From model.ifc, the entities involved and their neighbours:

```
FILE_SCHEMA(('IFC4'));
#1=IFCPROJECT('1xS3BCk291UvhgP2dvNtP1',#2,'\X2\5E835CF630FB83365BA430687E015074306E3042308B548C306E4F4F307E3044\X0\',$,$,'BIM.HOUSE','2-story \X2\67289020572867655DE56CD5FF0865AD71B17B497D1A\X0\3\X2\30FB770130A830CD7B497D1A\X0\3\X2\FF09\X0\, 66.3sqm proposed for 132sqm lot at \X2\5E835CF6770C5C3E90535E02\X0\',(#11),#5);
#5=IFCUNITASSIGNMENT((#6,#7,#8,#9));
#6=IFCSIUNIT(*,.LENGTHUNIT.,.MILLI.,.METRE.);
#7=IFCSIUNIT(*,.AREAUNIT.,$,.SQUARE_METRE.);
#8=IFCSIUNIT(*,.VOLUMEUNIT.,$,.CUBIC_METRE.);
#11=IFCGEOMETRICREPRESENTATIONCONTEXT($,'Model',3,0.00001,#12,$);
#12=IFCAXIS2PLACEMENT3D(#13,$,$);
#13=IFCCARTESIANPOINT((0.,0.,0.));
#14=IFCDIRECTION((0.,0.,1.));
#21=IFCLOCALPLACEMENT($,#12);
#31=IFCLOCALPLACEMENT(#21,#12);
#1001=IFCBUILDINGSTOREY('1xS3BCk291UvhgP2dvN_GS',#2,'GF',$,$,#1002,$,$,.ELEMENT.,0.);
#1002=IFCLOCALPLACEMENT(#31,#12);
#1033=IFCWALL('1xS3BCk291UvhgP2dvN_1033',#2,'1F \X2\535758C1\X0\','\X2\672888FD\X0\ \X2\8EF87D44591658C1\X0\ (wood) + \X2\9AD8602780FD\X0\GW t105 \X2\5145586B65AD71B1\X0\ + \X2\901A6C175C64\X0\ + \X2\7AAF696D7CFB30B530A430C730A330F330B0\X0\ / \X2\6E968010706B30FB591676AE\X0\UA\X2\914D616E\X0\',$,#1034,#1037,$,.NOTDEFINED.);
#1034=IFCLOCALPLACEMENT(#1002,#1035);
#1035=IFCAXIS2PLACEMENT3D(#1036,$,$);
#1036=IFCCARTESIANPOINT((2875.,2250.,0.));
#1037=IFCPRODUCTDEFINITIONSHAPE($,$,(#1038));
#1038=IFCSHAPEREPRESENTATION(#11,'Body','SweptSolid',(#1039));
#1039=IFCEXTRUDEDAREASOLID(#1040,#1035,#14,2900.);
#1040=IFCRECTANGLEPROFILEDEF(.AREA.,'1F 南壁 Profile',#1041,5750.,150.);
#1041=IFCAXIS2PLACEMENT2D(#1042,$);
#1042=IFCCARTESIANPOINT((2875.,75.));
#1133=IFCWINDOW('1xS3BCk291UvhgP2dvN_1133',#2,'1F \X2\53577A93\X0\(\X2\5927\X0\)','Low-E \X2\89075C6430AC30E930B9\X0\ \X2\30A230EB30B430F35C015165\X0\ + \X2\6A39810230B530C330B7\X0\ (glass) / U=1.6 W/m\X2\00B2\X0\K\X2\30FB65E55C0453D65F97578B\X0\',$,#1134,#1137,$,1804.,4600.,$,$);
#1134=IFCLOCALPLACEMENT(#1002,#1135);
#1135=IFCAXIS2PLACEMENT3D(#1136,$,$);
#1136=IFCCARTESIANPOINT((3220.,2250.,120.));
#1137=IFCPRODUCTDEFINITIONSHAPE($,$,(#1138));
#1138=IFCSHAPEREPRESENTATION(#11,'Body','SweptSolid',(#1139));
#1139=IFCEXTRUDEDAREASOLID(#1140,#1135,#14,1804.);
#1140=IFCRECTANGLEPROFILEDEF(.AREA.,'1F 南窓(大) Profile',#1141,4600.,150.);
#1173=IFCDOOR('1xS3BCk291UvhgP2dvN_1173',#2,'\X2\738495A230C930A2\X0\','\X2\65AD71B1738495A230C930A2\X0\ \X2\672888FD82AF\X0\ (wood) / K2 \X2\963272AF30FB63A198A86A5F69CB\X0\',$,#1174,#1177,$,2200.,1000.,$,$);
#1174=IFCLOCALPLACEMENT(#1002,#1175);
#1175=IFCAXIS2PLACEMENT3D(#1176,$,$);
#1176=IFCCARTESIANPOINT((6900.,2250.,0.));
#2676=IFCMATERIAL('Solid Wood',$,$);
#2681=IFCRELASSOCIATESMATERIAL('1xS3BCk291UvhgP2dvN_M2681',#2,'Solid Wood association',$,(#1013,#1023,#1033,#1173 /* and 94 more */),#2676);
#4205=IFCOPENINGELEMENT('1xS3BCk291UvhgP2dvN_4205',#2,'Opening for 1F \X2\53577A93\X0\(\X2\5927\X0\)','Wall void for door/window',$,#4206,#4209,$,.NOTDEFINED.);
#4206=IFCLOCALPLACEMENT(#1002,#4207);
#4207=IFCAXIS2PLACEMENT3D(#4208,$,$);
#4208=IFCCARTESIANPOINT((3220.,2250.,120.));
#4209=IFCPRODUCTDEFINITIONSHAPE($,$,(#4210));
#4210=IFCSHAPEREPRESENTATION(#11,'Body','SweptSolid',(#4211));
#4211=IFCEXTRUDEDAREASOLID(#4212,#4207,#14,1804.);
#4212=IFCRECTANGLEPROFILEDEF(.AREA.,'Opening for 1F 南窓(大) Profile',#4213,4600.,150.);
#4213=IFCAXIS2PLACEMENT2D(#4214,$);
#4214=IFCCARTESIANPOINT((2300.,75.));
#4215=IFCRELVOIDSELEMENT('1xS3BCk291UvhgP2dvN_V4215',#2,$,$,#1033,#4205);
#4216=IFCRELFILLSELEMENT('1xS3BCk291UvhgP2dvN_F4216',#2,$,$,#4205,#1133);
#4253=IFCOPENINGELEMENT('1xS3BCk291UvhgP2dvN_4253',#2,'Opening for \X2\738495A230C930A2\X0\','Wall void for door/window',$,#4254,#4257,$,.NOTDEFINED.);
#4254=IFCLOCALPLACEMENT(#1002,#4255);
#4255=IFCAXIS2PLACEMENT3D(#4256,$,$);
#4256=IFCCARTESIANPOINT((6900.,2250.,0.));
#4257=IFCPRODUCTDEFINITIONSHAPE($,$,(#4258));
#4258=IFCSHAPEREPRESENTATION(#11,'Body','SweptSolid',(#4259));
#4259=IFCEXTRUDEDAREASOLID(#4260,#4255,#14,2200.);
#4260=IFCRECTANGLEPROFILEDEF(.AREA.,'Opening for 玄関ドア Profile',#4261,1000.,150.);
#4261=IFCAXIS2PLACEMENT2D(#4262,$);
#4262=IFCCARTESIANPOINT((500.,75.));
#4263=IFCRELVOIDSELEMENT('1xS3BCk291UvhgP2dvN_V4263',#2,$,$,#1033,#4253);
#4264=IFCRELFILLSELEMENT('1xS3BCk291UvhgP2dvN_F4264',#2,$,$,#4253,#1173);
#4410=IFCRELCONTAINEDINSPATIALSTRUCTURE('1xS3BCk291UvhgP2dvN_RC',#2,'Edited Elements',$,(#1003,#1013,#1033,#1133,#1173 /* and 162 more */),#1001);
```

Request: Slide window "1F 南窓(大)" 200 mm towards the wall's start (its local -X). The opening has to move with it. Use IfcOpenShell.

```python
import ifcopenshell
import ifcopenshell.api.geometry
import ifcopenshell.util.placement
import ifcopenshell.util.unit

model = ifcopenshell.open("model.ifc")
unit_scale = ifcopenshell.util.unit.calculate_unit_scale(model)

window = model.by_guid("1xS3BCk291UvhgP2dvN_1133")
opening = window.FillsVoids[0].RelatingOpeningElement
wall = opening.VoidsElements[0].RelatingBuildingElement

wall_matrix = ifcopenshell.util.placement.get_local_placement(wall.ObjectPlacement)
shift = wall_matrix[:3, 0] * -0.2 / unit_scale
before = ifcopenshell.util.placement.get_local_placement(window.ObjectPlacement)[:3, 3].copy()

# The window is not placed relative to its opening, so move both.
for product in (opening, window):
    matrix = ifcopenshell.util.placement.get_local_placement(product.ObjectPlacement)
    matrix[:3, 3] += shift
    ifcopenshell.api.geometry.edit_object_placement(model, product=product, matrix=matrix, is_si=False)

after = ifcopenshell.util.placement.get_local_placement(window.ObjectPlacement)[:3, 3]
print("window moved by", (after - before).round(3) + 0.0)

model.write("model_v2.ifc")
```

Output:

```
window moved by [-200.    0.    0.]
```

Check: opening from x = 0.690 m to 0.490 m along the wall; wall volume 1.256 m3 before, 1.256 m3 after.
